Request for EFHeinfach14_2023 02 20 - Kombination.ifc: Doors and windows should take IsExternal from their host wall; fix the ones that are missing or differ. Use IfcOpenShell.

First a look at what the model holds.

```python
import ifcopenshell
import ifcopenshell.util.element

model = ifcopenshell.open("EFHeinfach14_2023 02 20 - Kombination.ifc")
print(model.schema)
seen = {}
for e in model.by_type("IfcDoor") + model.by_type("IfcWindow"):
    if not e.FillsVoids:
        continue
    host = e.FillsVoids[0].RelatingOpeningElement.VoidsElements[0].RelatingBuildingElement
    own = ifcopenshell.util.element.get_pset(e, f"Pset_{e.is_a()[3:].removesuffix('StandardCase')}Common", "IsExternal")
    wall = ifcopenshell.util.element.get_pset(host, "Pset_WallCommon", "IsExternal")
    seen[e.is_a(), own, wall] = seen.get((e.is_a(), own, wall), 0) + 1
for (cls, own, wall), count in sorted(seen.items(), key=str):
    print(count, cls, "IsExternal:", own, "| host wall:", wall)
```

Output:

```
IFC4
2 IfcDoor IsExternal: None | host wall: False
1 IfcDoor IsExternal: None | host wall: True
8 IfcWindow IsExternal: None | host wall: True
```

```python
import ifcopenshell
import ifcopenshell.api.pset
import ifcopenshell.util.element

model = ifcopenshell.open("EFHeinfach14_2023 02 20 - Kombination.ifc")

count = 0
for ifc_class, pset_name in (("IfcDoor", "Pset_DoorCommon"), ("IfcWindow", "Pset_WindowCommon")):
    for e in model.by_type(ifc_class):
        if not e.FillsVoids:
            continue
        host = e.FillsVoids[0].RelatingOpeningElement.VoidsElements[0].RelatingBuildingElement
        external = ifcopenshell.util.element.get_pset(host, "Pset_WallCommon", "IsExternal")
        if external is None or ifcopenshell.util.element.get_pset(e, pset_name, "IsExternal") == external:
            continue
        pset = ifcopenshell.api.pset.add_pset(model, product=e, name=pset_name)
        ifcopenshell.api.pset.edit_pset(model, pset=pset, properties={"IsExternal": external})
        count += 1

print(count, "updated")

model.write("EFHeinfach14_2023 02 20 - Kombination-out.ifc")
```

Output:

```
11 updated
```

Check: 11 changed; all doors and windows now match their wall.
